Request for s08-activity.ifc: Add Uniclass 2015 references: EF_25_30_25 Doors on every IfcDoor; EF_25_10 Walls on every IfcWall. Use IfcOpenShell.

First a look at what the model holds.

```python
import ifcopenshell

model = ifcopenshell.open("s08-activity.ifc")
print(model.schema)
print("classifications:", [c.Name for c in model.by_type("IfcClassification")])
for ifc_class in ("IfcDoor", "IfcRoof", "IfcStair", "IfcWall", "IfcWindow"):
    print(ifc_class, len(model.by_type(ifc_class)))
```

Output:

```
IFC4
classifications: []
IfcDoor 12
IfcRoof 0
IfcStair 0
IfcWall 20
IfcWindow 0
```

```python
import ifcopenshell
import ifcopenshell.api.classification

model = ifcopenshell.open("s08-activity.ifc")

system = ifcopenshell.api.classification.add_classification(model, classification="Uniclass 2015")

codes = {
    "IfcDoor": ("EF_25_30_25", "Doors"),
    "IfcWall": ("EF_25_10", "Walls"),
}
for ifc_class, (code, name) in codes.items():
    products = model.by_type(ifc_class)
    ifcopenshell.api.classification.add_reference(
        model, products=products, classification=system, identification=code, name=name
    )
    print(code, len(products))

model.write("s08-activity_updated.ifc")
```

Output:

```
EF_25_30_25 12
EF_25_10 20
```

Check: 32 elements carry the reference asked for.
